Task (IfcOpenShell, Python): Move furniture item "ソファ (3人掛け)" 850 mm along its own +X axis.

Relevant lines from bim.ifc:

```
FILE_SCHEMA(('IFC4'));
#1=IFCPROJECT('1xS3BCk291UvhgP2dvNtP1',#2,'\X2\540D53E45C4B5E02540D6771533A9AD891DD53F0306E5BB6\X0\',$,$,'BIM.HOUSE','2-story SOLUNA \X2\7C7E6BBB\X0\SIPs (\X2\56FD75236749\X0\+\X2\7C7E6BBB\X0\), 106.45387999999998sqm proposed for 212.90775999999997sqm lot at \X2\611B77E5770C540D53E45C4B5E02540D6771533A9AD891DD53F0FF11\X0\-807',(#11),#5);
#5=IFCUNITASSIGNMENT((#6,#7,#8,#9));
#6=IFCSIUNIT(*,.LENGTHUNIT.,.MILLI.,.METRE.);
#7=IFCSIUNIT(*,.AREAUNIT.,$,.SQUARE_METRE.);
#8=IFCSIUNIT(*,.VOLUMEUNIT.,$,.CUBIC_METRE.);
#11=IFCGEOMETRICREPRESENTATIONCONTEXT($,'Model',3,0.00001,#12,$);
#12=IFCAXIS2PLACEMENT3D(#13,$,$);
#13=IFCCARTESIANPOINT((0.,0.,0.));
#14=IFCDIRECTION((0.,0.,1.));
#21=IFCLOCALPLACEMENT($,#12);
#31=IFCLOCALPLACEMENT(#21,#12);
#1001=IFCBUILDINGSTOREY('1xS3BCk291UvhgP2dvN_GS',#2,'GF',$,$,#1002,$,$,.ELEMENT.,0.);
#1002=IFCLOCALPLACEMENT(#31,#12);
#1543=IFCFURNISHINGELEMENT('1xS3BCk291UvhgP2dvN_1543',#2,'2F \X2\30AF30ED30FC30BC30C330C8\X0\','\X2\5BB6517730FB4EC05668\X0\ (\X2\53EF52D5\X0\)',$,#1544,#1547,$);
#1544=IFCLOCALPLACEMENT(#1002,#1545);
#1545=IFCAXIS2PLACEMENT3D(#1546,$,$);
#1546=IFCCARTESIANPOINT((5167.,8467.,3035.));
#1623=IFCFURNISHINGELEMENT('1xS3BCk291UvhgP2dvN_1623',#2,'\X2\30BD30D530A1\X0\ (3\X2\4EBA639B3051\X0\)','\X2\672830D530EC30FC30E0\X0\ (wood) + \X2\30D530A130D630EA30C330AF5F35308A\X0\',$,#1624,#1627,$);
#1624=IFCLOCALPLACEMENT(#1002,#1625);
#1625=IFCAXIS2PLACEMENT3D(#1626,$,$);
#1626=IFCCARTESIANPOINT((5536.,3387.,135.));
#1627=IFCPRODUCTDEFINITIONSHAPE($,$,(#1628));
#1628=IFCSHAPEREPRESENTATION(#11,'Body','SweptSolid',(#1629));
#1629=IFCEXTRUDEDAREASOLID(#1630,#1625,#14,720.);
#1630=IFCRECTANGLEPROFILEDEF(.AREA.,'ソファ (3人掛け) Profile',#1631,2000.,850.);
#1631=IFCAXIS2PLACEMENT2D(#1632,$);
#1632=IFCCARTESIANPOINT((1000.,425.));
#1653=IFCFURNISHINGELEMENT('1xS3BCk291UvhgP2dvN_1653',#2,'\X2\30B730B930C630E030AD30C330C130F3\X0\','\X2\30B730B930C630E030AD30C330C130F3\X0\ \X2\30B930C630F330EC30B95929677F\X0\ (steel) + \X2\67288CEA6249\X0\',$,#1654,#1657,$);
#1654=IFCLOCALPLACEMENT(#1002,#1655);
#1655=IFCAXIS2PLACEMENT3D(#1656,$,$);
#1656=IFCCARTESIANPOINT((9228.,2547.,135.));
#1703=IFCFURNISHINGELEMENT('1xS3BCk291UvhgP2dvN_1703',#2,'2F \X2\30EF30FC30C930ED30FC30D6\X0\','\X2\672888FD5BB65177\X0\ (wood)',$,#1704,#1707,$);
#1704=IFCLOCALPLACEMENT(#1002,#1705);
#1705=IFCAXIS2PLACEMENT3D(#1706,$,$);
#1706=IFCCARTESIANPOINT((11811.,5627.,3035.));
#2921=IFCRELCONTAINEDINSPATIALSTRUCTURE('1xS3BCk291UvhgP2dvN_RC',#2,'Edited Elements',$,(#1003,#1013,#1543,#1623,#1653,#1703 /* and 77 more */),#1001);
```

```python
import ifcopenshell
import ifcopenshell.api.geometry
import ifcopenshell.util.placement
import ifcopenshell.util.unit

model = ifcopenshell.open("bim.ifc")
unit_scale = ifcopenshell.util.unit.calculate_unit_scale(model)

item = model.by_guid("1xS3BCk291UvhgP2dvN_1623")
matrix = ifcopenshell.util.placement.get_local_placement(item.ObjectPlacement)
matrix[:3, 3] += matrix[:3, 0] * 0.85 / unit_scale
ifcopenshell.api.geometry.edit_object_placement(model, product=item, matrix=matrix, is_si=False)

print(ifcopenshell.util.placement.get_local_placement(item.ObjectPlacement).round(3) + 0.0)

model.write("bim_v2.ifc")
```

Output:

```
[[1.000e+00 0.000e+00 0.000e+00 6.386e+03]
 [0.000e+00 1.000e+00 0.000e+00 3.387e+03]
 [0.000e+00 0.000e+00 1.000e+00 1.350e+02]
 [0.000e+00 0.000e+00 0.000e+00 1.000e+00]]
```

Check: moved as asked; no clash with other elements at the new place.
